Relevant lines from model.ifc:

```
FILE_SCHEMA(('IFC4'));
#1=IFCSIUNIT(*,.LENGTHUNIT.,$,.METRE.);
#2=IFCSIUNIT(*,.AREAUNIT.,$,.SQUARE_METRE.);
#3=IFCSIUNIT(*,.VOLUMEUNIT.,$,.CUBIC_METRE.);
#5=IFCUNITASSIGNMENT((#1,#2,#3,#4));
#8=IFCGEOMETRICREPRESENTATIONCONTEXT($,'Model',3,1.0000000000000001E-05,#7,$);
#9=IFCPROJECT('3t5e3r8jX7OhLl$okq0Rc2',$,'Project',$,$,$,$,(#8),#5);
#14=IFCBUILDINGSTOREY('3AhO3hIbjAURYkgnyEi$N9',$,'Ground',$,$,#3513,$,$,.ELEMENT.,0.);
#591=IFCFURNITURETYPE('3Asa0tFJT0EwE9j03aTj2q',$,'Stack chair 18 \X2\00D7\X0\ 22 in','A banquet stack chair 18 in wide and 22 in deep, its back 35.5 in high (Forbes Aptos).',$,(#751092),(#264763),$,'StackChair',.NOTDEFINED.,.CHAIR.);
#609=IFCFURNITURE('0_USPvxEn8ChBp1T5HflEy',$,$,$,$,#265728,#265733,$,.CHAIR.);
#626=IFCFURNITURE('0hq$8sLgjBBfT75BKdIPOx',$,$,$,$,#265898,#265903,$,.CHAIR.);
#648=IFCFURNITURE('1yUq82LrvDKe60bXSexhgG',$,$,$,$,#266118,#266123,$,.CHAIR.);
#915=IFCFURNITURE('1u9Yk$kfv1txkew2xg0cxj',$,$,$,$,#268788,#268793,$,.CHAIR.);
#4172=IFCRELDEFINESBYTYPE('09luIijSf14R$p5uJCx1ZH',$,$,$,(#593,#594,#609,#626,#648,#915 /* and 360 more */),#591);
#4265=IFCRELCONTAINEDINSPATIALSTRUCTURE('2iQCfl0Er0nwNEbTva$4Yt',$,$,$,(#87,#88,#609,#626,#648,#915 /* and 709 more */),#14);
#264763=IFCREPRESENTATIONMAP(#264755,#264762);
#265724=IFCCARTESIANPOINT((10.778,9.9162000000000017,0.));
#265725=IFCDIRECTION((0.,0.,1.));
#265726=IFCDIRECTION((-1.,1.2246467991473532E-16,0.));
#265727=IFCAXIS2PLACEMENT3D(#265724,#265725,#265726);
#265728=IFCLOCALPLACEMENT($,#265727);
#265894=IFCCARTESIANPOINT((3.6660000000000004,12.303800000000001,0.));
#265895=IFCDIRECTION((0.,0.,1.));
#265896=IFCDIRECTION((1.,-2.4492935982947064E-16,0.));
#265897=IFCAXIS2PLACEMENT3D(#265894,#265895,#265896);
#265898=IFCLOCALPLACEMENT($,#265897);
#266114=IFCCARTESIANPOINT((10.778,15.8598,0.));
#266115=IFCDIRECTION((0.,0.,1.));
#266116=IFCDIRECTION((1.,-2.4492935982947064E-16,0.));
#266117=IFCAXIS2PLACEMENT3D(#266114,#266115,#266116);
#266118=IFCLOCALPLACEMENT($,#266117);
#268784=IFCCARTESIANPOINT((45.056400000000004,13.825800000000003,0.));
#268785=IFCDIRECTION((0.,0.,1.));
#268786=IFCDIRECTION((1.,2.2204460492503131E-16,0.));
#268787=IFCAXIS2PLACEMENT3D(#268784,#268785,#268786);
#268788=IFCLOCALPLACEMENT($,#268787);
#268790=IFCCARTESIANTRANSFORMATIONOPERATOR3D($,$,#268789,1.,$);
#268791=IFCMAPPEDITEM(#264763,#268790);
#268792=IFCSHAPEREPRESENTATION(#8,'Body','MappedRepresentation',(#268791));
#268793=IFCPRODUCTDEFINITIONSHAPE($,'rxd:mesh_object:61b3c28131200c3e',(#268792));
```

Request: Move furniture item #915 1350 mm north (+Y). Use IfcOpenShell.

```python
import ifcopenshell
import ifcopenshell.api.geometry
import ifcopenshell.util.placement

model = ifcopenshell.open("model.ifc")

item = model.by_guid("1u9Yk$kfv1txkew2xg0cxj")
matrix = ifcopenshell.util.placement.get_local_placement(item.ObjectPlacement)
matrix[1, 3] += 1.35
ifcopenshell.api.geometry.edit_object_placement(model, product=item, matrix=matrix, is_si=False)

print(ifcopenshell.util.placement.get_local_placement(item.ObjectPlacement).round(3) + 0.0)

model.write("model-out.ifc")
```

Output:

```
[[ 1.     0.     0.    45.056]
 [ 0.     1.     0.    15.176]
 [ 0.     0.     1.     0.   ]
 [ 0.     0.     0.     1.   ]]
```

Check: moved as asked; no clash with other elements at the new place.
